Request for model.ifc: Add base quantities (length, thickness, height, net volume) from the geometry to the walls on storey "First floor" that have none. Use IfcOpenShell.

First a look at what the model holds.

```python
import ifcopenshell
import ifcopenshell.util.element
import ifcopenshell.util.unit

model = ifcopenshell.open("model.ifc")
print(model.schema)
for unit_type in ("LENGTHUNIT", "AREAUNIT", "VOLUMEUNIT"):
    print(unit_type, ifcopenshell.util.unit.calculate_unit_scale(model, unit_type))
storey = next(s for s in model.by_type("IfcBuildingStorey") if s.Name == "First floor")
walls = [e for e in ifcopenshell.util.element.get_decomposition(storey) if e.is_a("IfcWall")]
for e in sorted(walls, key=lambda e: e.id()):
    print(e.id(), e.is_a(), e.Name, list(ifcopenshell.util.element.get_psets(e, qtos_only=True)), sep=" | ")
```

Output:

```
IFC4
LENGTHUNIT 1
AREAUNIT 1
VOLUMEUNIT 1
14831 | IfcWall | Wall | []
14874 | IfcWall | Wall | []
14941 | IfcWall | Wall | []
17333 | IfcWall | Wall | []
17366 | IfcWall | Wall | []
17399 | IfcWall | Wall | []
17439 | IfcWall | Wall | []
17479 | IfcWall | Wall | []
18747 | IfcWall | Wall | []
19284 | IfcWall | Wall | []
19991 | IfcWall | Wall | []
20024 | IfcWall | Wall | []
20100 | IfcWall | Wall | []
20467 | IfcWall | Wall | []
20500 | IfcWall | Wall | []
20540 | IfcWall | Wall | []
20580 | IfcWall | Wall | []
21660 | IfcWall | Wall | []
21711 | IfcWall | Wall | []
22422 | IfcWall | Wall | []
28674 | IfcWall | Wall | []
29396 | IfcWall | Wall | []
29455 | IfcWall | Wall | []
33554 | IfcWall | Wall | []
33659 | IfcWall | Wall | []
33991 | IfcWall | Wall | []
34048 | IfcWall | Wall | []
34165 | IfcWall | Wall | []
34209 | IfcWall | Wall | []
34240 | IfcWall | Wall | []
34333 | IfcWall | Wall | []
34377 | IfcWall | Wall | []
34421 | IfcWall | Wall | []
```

```python
import ifcopenshell
import ifcopenshell.api.pset
import ifcopenshell.geom
import ifcopenshell.util.element
import ifcopenshell.util.shape
import ifcopenshell.util.unit

model = ifcopenshell.open("model.ifc")
unit_scale = ifcopenshell.util.unit.calculate_unit_scale(model)
volume_scale = ifcopenshell.util.unit.calculate_unit_scale(model, "VOLUMEUNIT")
settings = ifcopenshell.geom.settings()

storey = next(s for s in model.by_type("IfcBuildingStorey") if s.Name == "First floor")
walls = [e for e in ifcopenshell.util.element.get_decomposition(storey) if e.is_a("IfcWall")]

for e in sorted(walls, key=lambda e: e.id()):
    if ifcopenshell.util.element.get_psets(e, qtos_only=True, should_inherit=False):
        continue
    # Geometry comes back in metres, in the element's own axes.
    shape = ifcopenshell.geom.create_shape(settings, e)
    values = {
        "Length": ifcopenshell.util.shape.get_x(shape.geometry) / unit_scale,
        "Width": ifcopenshell.util.shape.get_y(shape.geometry) / unit_scale,
        "Height": ifcopenshell.util.shape.get_z(shape.geometry) / unit_scale,
        "NetVolume": ifcopenshell.util.shape.get_volume(shape.geometry) / volume_scale,
    }
    qto = ifcopenshell.api.pset.add_qto(model, product=e, name="Qto_WallBaseQuantities")
    ifcopenshell.api.pset.edit_qto(model, qto=qto, properties=values)
    print(e.id(), {k: round(v, 3) for k, v in values.items()})

model.write("model_v2.ifc")
```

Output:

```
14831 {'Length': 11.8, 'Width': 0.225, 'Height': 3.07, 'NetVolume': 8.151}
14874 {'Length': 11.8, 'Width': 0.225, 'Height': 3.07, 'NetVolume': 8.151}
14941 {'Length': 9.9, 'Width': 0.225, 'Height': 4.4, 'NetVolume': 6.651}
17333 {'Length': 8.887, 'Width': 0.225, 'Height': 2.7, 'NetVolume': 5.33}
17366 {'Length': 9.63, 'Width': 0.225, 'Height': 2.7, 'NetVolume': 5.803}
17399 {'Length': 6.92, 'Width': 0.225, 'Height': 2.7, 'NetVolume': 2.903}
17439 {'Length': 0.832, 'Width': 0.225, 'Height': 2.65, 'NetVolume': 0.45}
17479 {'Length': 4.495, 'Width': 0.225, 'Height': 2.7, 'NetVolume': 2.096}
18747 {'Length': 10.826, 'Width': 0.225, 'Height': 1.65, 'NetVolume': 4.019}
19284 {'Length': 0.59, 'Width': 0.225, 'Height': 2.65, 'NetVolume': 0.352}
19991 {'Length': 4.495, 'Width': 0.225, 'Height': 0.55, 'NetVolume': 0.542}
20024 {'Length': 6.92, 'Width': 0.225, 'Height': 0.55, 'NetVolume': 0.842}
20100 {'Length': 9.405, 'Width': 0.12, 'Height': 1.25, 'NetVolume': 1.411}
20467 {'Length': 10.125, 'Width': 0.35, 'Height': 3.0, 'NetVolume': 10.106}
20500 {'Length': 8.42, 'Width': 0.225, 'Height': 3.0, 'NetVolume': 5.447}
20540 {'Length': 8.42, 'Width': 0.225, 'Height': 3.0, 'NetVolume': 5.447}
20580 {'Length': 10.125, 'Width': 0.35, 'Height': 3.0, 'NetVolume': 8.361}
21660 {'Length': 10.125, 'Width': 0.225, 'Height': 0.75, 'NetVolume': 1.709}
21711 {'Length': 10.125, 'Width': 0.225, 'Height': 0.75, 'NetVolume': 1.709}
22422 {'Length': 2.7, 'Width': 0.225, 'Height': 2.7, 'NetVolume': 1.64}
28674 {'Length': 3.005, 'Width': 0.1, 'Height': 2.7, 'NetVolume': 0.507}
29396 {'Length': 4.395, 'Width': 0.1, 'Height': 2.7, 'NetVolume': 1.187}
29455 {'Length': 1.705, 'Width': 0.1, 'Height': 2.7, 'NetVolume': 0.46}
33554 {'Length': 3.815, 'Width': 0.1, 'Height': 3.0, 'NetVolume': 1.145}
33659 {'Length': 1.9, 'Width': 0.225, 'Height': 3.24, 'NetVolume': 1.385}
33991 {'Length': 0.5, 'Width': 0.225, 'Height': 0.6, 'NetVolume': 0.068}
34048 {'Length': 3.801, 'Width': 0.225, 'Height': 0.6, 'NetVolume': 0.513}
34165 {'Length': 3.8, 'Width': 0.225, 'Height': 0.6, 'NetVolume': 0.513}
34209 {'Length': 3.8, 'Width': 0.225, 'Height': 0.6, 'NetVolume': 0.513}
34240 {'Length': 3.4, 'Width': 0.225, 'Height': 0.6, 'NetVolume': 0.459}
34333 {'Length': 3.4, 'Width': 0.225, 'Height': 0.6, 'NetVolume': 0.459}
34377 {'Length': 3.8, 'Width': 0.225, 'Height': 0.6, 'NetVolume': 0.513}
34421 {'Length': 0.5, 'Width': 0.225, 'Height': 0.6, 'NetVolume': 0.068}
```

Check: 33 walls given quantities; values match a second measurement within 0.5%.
